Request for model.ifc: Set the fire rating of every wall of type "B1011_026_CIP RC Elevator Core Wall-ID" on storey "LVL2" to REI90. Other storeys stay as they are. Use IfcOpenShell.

First a look at what the model holds.

```python
import ifcopenshell
import ifcopenshell.util.element

model = ifcopenshell.open("model.ifc")
print(model.schema)
storey = next(s for s in model.by_type("IfcBuildingStorey") if s.Name == "LVL2")
walls = [e for e in ifcopenshell.util.element.get_decomposition(storey) if e.is_a("IfcWall")]
seen = {}
for e in walls:
    element_type = ifcopenshell.util.element.get_type(e)
    key = (element_type.Name if element_type != e and element_type else None, ifcopenshell.util.element.get_pset(e, "Pset_WallCommon", "FireRating"))
    seen[key] = seen.get(key, 0) + 1
for (name, value), count in sorted(seen.items(), key=str):
    print(count, "x", name, "|", value)
```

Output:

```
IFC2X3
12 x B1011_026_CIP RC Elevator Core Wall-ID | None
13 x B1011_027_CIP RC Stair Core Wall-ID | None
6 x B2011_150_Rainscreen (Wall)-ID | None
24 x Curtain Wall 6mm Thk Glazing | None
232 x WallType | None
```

```python
import ifcopenshell
import ifcopenshell.api.pset
import ifcopenshell.util.element

model = ifcopenshell.open("model.ifc")

storey = next(s for s in model.by_type("IfcBuildingStorey") if s.Name == "LVL2")
walls = [e for e in ifcopenshell.util.element.get_decomposition(storey) if e.is_a("IfcWall")]

count = 0
for e in walls:
    element_type = ifcopenshell.util.element.get_type(e)
    if element_type in (None, e) or element_type.Name != "B1011_026_CIP RC Elevator Core Wall-ID":
        continue
    found = ifcopenshell.util.element.get_pset(e, "Pset_WallCommon", should_inherit=False)
    if found:
        pset = model.by_id(found["id"])
        if len(ifcopenshell.util.element.get_elements_by_pset(pset)) > 1:
            pset = ifcopenshell.api.pset.unshare_pset(model, products=[e], pset=pset)[0]
    else:
        pset = ifcopenshell.api.pset.add_pset(model, product=e, name="Pset_WallCommon")
    ifcopenshell.api.pset.edit_pset(model, pset=pset, properties={"FireRating": "REI90"})
    count += 1

print(count, "walls updated")

model.write("model_v2.ifc")
```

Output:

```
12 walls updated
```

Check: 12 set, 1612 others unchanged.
